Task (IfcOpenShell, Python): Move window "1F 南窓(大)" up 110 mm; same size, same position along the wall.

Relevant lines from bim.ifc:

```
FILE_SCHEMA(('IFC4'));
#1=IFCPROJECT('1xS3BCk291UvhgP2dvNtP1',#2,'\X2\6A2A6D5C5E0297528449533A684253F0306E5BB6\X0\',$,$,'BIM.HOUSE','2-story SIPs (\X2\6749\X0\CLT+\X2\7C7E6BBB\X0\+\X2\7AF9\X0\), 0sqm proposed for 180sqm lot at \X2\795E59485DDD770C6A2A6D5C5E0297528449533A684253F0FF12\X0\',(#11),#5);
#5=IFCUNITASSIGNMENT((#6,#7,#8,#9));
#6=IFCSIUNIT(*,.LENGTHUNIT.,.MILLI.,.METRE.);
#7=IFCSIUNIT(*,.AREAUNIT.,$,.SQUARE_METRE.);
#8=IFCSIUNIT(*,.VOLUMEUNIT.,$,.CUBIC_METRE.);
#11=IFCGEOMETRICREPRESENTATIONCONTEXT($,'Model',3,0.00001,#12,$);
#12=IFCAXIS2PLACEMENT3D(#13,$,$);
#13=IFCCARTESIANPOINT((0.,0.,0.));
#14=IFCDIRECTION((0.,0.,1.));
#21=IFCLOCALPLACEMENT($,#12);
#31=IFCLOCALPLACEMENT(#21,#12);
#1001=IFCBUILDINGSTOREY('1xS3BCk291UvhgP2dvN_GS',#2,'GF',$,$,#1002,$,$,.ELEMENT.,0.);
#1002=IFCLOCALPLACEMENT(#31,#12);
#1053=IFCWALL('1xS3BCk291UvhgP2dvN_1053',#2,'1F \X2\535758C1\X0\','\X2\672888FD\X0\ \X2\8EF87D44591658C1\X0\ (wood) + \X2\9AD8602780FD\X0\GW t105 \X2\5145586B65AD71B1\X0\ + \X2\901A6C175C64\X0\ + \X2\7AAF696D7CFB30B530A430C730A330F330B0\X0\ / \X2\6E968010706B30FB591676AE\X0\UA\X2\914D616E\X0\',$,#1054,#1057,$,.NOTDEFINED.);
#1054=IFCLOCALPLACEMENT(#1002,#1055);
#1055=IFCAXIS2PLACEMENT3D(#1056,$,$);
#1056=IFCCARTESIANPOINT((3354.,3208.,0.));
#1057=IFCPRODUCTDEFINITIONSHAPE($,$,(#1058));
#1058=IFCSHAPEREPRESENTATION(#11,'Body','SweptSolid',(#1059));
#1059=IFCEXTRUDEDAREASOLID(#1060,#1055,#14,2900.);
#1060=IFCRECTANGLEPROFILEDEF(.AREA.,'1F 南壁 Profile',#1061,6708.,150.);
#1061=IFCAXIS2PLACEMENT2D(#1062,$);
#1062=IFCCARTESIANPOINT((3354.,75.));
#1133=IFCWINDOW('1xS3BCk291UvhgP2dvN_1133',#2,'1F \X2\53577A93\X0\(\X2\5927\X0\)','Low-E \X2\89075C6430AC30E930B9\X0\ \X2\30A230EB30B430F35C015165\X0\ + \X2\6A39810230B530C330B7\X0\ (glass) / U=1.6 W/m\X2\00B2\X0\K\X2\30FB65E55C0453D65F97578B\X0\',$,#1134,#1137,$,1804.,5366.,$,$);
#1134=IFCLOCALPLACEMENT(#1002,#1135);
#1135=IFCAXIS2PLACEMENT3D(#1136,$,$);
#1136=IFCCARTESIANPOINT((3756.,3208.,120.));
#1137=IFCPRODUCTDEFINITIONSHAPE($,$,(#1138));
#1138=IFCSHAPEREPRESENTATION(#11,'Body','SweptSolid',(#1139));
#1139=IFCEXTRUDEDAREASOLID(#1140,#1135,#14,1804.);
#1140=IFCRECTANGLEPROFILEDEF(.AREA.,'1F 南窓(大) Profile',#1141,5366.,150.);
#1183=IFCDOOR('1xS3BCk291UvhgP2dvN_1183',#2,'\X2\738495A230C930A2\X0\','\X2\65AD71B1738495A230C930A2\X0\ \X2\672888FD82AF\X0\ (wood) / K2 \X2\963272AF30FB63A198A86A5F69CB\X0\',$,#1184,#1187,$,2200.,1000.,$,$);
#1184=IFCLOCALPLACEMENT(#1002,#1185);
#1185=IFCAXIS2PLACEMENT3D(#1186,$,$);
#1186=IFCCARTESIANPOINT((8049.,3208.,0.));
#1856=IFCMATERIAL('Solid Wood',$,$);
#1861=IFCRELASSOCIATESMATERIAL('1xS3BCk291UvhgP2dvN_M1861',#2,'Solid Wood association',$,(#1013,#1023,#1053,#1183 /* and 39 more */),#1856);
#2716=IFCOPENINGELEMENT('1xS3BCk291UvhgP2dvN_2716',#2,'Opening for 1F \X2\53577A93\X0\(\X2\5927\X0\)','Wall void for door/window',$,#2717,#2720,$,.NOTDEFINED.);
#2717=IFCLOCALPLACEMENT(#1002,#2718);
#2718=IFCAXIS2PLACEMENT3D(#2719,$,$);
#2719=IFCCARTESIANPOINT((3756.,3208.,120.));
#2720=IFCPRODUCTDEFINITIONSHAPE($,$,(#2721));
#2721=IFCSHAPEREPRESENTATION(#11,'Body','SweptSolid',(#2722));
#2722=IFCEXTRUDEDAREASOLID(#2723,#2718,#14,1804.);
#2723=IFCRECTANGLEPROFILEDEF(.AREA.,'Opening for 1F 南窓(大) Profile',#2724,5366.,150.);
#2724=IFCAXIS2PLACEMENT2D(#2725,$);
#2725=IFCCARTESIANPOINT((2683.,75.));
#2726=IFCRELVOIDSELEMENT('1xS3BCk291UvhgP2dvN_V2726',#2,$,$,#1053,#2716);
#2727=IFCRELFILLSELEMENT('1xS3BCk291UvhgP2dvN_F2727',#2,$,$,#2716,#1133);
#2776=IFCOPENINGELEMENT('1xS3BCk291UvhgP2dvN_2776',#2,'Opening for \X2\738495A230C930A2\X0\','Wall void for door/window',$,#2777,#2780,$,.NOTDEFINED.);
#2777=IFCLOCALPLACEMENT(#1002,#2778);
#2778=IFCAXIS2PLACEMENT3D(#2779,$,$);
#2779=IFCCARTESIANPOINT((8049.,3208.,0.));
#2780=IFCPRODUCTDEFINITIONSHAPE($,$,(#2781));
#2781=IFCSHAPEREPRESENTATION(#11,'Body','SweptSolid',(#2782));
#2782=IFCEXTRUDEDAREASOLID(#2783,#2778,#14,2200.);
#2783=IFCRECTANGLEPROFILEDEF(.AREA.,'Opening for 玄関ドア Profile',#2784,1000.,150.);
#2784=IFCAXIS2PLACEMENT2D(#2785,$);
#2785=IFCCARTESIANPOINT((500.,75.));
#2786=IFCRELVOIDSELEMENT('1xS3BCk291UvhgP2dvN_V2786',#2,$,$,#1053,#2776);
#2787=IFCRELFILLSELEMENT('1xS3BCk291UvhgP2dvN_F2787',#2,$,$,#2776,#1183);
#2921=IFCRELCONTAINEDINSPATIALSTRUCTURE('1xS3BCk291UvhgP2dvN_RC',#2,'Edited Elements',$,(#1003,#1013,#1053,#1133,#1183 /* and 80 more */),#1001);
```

```python
import numpy as np
import ifcopenshell
import ifcopenshell.api.geometry
import ifcopenshell.util.placement
import ifcopenshell.util.unit

model = ifcopenshell.open("bim.ifc")
unit_scale = ifcopenshell.util.unit.calculate_unit_scale(model)

window = model.by_id(1133)
opening = window.FillsVoids[0].RelatingOpeningElement
dz = 0.11 / unit_scale

shift = np.array([0.0, 0.0, dz])
# The window is not placed relative to its opening, so move both.
for product in (opening, window):
    matrix = ifcopenshell.util.placement.get_local_placement(product.ObjectPlacement)
    matrix[:3, 3] += shift
    ifcopenshell.api.geometry.edit_object_placement(model, product=product, matrix=matrix, is_si=False)

print(f"moved by {dz * unit_scale:+.3f} m")

model.write("bim_edited.ifc")
```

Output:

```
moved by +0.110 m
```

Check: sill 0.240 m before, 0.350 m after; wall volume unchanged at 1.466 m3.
